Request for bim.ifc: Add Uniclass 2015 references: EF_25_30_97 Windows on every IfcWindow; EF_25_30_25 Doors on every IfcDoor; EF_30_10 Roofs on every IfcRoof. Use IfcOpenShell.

First a look at what the model holds.

```python
import ifcopenshell

model = ifcopenshell.open("bim.ifc")
print(model.schema)
print("classifications:", [c.Name for c in model.by_type("IfcClassification")])
for ifc_class in ("IfcDoor", "IfcRoof", "IfcStair", "IfcWall", "IfcWindow"):
    print(ifc_class, len(model.by_type(ifc_class)))
```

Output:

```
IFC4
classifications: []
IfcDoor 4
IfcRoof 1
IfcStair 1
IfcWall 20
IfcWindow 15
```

```python
import ifcopenshell
import ifcopenshell.api.classification

model = ifcopenshell.open("bim.ifc")

system = ifcopenshell.api.classification.add_classification(model, classification="Uniclass 2015")

codes = {
    "IfcWindow": ("EF_25_30_97", "Windows"),
    "IfcDoor": ("EF_25_30_25", "Doors"),
    "IfcRoof": ("EF_30_10", "Roofs"),
}
for ifc_class, (code, name) in codes.items():
    products = model.by_type(ifc_class)
    ifcopenshell.api.classification.add_reference(
        model, products=products, classification=system, identification=code, name=name
    )
    print(code, len(products))

model.write("bim-out.ifc")
```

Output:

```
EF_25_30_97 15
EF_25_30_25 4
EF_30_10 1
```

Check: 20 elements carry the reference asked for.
